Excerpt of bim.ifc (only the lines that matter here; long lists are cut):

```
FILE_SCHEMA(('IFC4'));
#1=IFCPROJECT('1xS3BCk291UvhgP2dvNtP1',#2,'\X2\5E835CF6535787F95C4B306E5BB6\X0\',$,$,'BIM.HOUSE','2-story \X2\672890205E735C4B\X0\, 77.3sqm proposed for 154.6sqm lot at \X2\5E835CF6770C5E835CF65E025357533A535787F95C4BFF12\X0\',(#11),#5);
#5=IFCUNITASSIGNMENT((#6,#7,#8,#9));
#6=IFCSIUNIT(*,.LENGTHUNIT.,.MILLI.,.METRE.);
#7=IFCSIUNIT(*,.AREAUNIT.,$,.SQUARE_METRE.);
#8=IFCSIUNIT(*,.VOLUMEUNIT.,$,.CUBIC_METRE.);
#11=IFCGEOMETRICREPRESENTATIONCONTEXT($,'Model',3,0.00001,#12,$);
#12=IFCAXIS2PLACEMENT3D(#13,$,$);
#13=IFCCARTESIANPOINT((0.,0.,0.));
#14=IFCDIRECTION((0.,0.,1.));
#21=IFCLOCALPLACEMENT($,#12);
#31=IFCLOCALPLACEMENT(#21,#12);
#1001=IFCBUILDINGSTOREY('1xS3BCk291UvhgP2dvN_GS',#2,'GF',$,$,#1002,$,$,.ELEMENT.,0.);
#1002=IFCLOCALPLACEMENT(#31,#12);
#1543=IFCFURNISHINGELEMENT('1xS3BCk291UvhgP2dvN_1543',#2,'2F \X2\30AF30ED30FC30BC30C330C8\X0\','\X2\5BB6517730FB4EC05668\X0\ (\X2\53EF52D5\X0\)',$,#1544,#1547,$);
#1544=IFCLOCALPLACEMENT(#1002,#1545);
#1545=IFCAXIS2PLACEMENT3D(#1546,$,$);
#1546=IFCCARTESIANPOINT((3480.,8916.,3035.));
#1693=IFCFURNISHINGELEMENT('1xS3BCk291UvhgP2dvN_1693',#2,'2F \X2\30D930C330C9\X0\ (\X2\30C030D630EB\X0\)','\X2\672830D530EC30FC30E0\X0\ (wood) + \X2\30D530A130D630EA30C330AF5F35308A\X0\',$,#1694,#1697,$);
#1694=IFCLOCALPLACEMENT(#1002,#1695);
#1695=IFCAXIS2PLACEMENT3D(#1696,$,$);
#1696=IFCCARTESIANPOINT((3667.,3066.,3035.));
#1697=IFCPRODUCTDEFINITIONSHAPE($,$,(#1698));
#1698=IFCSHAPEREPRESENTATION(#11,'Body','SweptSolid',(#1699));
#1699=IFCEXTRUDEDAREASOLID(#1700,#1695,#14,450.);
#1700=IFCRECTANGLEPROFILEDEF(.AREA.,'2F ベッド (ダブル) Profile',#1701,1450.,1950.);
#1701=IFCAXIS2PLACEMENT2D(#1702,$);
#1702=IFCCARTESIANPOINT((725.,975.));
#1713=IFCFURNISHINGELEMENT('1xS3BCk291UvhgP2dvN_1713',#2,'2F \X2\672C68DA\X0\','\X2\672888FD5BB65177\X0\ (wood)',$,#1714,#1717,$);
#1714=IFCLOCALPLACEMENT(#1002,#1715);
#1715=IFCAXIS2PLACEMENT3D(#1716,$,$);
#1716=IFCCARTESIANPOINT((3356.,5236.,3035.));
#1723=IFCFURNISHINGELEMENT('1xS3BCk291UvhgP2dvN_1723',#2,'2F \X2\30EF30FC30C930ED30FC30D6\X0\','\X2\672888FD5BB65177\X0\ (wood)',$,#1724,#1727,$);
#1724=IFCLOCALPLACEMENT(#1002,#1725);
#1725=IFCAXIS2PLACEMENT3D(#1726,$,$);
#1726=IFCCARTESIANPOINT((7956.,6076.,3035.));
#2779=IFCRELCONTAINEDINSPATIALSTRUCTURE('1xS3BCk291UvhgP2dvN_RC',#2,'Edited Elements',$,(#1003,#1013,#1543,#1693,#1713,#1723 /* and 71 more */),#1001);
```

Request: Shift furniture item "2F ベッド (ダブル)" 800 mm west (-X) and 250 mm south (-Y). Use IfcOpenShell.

```python
import ifcopenshell
import ifcopenshell.api.geometry
import ifcopenshell.util.placement

model = ifcopenshell.open("bim.ifc")

item = model.by_id(1693)
matrix = ifcopenshell.util.placement.get_local_placement(item.ObjectPlacement)
matrix[0, 3] -= 800.0
matrix[1, 3] -= 250.0
ifcopenshell.api.geometry.edit_object_placement(model, product=item, matrix=matrix, is_si=False)

print(ifcopenshell.util.placement.get_local_placement(item.ObjectPlacement).round(3) + 0.0)

model.write("bim_rev.ifc")
```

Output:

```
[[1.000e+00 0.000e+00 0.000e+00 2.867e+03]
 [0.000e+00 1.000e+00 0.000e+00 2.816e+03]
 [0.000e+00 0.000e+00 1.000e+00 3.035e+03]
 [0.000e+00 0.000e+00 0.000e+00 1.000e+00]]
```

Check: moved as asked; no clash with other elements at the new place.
